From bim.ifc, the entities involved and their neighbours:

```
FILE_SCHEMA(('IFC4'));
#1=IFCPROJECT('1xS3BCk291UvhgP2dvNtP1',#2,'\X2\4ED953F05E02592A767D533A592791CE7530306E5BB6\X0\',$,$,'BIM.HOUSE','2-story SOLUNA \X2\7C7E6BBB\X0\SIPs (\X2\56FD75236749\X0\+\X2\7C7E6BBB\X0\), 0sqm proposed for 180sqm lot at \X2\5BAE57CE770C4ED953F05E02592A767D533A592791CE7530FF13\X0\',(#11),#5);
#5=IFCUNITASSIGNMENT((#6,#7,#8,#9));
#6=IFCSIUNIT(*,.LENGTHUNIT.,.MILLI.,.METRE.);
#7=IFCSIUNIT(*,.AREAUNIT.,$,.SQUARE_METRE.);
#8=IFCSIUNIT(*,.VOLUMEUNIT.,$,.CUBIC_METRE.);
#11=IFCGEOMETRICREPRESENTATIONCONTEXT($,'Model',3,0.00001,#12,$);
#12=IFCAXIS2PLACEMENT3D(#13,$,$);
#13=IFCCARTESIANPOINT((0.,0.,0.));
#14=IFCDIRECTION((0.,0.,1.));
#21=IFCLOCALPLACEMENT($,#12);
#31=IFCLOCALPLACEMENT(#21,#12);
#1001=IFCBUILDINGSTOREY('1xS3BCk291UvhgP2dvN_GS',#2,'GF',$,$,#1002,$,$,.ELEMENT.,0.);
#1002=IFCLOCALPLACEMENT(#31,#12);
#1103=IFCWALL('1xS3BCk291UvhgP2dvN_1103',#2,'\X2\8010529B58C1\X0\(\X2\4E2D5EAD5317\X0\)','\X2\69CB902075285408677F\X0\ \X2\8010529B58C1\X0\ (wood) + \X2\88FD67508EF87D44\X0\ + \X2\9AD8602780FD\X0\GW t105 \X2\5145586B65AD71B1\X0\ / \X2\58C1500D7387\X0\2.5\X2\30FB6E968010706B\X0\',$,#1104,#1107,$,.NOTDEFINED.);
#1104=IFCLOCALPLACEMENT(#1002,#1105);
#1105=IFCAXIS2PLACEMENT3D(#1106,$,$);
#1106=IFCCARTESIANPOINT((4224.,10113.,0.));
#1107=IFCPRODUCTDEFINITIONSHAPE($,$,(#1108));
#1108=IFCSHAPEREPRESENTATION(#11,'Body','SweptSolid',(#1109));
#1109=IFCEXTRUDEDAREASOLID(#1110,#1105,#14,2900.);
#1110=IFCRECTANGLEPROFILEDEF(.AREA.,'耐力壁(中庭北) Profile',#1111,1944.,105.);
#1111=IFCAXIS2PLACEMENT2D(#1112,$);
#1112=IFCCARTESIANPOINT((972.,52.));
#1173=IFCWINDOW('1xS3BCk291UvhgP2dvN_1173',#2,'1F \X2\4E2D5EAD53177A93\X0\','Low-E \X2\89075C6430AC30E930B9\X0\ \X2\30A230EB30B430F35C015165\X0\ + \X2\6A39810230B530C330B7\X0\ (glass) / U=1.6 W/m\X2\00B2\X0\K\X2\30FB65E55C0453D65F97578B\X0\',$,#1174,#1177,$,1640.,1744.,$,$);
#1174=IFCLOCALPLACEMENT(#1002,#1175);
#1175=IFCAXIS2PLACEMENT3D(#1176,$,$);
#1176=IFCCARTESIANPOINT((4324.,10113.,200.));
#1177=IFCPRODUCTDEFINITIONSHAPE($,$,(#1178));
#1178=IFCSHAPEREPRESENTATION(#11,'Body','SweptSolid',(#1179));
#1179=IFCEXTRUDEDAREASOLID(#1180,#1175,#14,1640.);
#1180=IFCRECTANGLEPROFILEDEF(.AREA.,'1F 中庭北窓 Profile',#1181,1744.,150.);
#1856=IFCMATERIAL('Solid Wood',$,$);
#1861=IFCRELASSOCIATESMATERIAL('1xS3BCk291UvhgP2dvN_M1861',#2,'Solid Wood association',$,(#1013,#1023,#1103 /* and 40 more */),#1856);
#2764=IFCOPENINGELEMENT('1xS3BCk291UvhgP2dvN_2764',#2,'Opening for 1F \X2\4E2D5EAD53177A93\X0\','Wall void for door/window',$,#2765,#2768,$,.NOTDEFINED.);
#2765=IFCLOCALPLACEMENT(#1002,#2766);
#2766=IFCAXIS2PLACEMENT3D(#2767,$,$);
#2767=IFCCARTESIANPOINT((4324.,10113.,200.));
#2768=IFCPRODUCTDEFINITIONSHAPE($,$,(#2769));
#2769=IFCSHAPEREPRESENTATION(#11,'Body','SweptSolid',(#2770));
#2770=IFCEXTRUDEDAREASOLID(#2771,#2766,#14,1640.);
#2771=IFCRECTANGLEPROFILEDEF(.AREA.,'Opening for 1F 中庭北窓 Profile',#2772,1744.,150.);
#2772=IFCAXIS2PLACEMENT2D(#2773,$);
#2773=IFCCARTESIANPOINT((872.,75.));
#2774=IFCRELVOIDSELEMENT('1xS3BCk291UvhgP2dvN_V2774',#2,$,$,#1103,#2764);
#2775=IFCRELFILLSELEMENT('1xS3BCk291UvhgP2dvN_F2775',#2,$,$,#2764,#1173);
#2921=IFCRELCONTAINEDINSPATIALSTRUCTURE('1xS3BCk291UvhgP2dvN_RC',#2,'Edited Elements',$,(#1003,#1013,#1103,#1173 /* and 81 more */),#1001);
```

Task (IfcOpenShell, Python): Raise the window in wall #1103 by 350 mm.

```python
import numpy as np
import ifcopenshell
import ifcopenshell.api.geometry
import ifcopenshell.util.placement
import ifcopenshell.util.unit

model = ifcopenshell.open("bim.ifc")
unit_scale = ifcopenshell.util.unit.calculate_unit_scale(model)

window = model.by_guid("1xS3BCk291UvhgP2dvN_1173")
opening = window.FillsVoids[0].RelatingOpeningElement
dz = 0.35 / unit_scale

shift = np.array([0.0, 0.0, dz])
# The window is not placed relative to its opening, so move both.
for product in (opening, window):
    matrix = ifcopenshell.util.placement.get_local_placement(product.ObjectPlacement)
    matrix[:3, 3] += shift
    ifcopenshell.api.geometry.edit_object_placement(model, product=product, matrix=matrix, is_si=False)

print(f"moved by {dz * unit_scale:+.3f} m")

model.write("bim-out.ifc")
```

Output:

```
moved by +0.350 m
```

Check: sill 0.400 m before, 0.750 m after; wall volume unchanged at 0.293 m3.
